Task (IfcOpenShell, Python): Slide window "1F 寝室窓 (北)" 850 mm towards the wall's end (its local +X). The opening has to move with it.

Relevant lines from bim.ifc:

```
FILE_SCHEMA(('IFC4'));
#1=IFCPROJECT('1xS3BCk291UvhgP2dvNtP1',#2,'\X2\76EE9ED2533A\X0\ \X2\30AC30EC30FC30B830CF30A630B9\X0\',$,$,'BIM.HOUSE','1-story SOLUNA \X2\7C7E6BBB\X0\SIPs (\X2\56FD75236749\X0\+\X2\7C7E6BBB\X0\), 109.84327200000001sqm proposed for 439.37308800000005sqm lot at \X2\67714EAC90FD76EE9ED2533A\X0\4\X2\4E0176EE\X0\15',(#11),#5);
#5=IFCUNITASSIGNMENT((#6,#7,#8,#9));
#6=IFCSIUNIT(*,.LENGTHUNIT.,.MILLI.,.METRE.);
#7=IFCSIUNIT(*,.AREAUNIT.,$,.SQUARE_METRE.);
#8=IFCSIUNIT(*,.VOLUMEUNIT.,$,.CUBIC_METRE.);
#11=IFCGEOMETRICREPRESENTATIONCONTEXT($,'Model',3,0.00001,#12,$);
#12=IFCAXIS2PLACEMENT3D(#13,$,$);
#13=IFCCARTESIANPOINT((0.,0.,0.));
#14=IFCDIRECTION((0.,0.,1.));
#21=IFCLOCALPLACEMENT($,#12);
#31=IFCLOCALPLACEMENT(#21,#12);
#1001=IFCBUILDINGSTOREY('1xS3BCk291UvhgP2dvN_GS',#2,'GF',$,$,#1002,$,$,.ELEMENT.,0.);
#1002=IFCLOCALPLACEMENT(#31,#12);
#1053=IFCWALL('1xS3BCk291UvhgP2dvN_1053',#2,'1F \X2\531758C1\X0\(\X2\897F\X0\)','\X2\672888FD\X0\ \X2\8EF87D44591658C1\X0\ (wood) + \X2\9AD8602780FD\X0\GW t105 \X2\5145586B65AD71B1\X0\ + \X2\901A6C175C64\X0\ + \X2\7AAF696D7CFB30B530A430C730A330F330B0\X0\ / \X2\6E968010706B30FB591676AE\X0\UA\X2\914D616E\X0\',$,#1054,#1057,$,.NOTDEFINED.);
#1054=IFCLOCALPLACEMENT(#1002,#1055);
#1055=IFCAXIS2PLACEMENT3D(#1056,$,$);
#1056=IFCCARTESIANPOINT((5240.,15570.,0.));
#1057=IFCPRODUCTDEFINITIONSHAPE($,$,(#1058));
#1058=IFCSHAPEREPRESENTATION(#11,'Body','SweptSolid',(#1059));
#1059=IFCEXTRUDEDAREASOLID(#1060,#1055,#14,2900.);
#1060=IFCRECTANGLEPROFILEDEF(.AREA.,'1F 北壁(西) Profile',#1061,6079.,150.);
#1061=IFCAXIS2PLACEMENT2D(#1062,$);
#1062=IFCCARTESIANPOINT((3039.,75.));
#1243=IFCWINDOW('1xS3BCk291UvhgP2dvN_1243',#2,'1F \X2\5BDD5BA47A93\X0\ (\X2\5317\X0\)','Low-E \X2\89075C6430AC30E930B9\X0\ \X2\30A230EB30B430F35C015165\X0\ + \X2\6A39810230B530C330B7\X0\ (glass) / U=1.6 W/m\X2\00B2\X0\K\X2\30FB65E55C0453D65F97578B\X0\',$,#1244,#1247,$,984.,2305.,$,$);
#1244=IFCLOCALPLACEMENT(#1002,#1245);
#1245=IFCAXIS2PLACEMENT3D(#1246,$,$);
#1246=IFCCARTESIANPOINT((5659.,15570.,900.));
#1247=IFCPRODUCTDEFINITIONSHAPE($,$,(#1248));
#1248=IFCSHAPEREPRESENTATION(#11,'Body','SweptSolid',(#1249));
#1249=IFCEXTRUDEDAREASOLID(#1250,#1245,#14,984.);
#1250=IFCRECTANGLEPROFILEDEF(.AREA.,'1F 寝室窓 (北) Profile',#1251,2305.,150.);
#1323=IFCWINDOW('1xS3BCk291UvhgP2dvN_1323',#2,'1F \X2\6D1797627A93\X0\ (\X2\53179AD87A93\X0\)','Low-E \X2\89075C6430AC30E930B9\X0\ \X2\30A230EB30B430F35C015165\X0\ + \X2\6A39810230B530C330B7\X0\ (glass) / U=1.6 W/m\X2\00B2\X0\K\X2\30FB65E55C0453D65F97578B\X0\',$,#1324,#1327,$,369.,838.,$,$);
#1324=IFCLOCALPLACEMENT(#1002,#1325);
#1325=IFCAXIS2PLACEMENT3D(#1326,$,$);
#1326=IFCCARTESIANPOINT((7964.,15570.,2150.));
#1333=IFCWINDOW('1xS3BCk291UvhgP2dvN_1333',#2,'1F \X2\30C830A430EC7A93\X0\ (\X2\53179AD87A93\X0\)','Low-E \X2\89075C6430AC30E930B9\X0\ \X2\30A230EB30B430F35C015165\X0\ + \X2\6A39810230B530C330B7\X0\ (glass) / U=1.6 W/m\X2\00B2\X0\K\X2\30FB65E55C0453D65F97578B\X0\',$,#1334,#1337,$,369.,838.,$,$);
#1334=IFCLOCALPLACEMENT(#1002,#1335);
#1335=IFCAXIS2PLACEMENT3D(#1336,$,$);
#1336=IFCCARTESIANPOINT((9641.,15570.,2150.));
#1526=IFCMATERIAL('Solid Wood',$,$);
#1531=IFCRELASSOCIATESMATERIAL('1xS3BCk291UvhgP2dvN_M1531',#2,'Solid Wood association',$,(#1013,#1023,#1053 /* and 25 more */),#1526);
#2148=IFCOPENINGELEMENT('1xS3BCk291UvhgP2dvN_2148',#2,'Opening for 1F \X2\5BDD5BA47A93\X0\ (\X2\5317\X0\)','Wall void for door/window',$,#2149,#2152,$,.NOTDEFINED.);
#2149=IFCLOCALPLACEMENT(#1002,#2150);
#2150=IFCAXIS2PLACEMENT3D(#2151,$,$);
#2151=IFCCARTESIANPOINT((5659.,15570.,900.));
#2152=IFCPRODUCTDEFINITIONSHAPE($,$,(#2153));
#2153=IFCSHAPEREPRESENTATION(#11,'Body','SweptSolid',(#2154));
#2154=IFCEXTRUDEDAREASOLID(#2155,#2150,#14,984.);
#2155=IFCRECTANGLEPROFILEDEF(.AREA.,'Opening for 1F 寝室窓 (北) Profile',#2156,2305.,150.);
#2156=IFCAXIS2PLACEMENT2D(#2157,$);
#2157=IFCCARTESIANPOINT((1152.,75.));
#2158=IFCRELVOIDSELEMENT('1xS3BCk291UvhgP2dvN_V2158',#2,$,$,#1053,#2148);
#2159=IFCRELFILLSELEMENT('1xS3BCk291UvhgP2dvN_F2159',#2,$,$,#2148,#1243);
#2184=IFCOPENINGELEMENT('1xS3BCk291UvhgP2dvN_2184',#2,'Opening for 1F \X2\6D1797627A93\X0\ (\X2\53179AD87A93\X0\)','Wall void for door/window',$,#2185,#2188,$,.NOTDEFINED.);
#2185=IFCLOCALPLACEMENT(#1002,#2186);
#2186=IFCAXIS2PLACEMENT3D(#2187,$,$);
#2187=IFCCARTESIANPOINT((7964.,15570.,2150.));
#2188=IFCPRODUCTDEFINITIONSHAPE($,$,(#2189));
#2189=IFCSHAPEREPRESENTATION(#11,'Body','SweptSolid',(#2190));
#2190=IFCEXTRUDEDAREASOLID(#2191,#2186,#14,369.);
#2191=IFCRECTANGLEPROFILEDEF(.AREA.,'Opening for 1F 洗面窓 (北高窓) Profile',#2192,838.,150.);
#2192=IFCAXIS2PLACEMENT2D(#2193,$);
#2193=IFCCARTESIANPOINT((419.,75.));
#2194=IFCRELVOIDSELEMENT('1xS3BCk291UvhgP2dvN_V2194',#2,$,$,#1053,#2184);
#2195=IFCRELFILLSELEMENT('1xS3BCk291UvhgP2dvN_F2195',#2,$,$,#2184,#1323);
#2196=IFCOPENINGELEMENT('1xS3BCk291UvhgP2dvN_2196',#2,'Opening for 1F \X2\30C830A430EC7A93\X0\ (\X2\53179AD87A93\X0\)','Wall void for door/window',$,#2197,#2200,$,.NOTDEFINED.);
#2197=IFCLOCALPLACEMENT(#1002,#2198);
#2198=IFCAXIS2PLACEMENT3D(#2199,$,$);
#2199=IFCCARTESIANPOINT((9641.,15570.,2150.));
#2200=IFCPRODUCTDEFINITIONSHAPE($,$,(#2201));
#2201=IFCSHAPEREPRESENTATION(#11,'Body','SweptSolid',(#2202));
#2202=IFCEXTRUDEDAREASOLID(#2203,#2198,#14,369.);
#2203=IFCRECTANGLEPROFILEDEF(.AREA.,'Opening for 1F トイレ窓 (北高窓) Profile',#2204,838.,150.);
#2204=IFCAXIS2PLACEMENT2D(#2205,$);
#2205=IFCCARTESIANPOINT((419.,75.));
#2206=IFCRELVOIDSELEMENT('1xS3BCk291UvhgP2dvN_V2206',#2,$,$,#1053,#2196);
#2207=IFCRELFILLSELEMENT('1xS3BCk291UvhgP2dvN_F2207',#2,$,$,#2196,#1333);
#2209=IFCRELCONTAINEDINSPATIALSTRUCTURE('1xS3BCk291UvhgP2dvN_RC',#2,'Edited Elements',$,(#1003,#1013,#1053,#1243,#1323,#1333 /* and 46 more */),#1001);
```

```python
import ifcopenshell
import ifcopenshell.api.geometry
import ifcopenshell.util.placement
import ifcopenshell.util.unit

model = ifcopenshell.open("bim.ifc")
unit_scale = ifcopenshell.util.unit.calculate_unit_scale(model)

window = model.by_id(1243)
opening = window.FillsVoids[0].RelatingOpeningElement
wall = opening.VoidsElements[0].RelatingBuildingElement

wall_matrix = ifcopenshell.util.placement.get_local_placement(wall.ObjectPlacement)
shift = wall_matrix[:3, 0] * 0.85 / unit_scale
before = ifcopenshell.util.placement.get_local_placement(window.ObjectPlacement)[:3, 3].copy()

# The window is not placed relative to its opening, so move both.
for product in (opening, window):
    matrix = ifcopenshell.util.placement.get_local_placement(product.ObjectPlacement)
    matrix[:3, 3] += shift
    ifcopenshell.api.geometry.edit_object_placement(model, product=product, matrix=matrix, is_si=False)

after = ifcopenshell.util.placement.get_local_placement(window.ObjectPlacement)[:3, 3]
print("window moved by", (after - before).round(3) + 0.0)

model.write("bim_edited.ifc")
```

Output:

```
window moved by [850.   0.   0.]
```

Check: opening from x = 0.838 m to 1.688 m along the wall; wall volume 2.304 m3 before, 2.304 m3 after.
